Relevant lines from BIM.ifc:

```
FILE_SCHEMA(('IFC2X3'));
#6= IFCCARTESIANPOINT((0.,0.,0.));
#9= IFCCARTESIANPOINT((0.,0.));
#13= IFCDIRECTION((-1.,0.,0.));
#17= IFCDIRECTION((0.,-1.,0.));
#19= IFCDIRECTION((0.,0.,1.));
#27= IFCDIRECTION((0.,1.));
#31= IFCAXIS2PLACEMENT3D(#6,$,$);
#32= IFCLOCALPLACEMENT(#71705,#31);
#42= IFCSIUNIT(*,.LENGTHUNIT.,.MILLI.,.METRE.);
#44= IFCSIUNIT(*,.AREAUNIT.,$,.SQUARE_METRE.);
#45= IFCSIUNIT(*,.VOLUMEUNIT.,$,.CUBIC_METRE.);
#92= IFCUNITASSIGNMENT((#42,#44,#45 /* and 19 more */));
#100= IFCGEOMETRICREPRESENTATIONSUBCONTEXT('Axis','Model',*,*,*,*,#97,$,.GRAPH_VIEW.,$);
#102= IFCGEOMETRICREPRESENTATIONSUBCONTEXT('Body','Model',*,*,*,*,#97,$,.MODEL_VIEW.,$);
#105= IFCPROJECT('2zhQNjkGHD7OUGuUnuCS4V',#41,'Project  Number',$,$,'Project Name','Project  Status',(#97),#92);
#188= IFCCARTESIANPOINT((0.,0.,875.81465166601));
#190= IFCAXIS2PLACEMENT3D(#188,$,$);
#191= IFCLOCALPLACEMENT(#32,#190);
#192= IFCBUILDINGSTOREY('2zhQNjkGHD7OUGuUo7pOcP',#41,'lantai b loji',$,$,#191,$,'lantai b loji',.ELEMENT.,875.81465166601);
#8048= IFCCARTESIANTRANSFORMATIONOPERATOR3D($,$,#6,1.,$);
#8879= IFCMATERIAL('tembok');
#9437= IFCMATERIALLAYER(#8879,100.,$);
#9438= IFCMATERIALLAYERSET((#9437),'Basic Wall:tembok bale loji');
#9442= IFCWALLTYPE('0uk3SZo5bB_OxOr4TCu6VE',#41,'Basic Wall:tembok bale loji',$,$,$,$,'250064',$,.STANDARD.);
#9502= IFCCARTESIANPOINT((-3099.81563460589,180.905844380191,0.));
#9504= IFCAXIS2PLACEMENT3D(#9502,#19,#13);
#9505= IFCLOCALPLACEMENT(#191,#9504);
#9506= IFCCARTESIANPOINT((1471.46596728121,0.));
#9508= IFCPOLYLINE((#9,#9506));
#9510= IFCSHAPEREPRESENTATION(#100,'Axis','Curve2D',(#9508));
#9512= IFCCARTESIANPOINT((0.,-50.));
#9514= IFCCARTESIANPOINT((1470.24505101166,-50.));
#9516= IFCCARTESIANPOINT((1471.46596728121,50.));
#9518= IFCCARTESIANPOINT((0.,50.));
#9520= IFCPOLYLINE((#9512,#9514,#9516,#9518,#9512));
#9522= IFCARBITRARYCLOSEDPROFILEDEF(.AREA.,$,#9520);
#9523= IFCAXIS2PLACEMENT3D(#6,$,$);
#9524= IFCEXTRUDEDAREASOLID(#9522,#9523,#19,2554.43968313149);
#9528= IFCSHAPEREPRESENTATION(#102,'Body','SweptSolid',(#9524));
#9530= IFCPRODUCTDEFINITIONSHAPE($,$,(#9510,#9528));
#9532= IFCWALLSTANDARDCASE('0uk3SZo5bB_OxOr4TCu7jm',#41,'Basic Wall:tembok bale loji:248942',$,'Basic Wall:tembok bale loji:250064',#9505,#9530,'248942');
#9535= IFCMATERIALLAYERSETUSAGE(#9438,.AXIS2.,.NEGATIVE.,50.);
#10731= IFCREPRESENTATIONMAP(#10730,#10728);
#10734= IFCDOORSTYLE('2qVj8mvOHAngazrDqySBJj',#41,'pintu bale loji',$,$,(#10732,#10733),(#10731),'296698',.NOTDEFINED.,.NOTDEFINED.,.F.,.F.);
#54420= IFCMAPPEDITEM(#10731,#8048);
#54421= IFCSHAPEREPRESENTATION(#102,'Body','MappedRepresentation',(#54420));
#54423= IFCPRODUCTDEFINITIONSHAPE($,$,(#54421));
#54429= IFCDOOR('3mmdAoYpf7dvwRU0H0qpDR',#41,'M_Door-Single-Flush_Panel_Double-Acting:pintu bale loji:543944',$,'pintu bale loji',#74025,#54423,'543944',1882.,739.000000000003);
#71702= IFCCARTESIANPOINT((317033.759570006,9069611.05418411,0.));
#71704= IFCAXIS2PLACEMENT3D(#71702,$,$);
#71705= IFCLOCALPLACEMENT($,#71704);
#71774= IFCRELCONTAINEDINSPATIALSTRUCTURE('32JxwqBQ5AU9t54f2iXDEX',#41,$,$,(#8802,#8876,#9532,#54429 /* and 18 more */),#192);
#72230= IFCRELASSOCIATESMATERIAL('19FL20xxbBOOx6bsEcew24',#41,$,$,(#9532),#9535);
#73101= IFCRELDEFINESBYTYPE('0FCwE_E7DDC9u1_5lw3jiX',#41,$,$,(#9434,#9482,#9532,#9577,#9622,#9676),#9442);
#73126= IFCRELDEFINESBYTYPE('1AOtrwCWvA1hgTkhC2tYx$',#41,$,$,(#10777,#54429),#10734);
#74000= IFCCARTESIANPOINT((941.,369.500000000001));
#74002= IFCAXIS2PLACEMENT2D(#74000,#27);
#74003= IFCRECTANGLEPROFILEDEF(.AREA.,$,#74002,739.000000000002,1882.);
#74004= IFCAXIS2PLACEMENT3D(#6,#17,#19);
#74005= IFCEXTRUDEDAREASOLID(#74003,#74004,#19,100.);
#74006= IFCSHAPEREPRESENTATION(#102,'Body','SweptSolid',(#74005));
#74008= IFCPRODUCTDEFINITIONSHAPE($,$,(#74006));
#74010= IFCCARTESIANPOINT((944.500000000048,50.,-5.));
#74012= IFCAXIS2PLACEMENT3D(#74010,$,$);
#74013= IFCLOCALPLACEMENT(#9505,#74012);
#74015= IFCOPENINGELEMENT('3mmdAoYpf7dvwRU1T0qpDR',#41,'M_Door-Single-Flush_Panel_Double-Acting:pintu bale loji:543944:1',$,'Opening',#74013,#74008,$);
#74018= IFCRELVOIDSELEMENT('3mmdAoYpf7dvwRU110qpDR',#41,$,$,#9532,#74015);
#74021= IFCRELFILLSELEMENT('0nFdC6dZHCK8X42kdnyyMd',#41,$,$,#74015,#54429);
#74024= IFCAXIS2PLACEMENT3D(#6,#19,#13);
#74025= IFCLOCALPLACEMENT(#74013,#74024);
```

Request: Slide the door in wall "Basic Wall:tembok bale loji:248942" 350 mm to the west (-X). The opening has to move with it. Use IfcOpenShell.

```python
import ifcopenshell
import ifcopenshell.api.geometry
import ifcopenshell.util.placement
import ifcopenshell.util.unit

model = ifcopenshell.open("BIM.ifc")
unit_scale = ifcopenshell.util.unit.calculate_unit_scale(model)

door = model.by_id(54429)
opening = door.FillsVoids[0].RelatingOpeningElement
wall = opening.VoidsElements[0].RelatingBuildingElement

wall_matrix = ifcopenshell.util.placement.get_local_placement(wall.ObjectPlacement)
shift = wall_matrix[:3, 0] * 0.35 / unit_scale
before = ifcopenshell.util.placement.get_local_placement(door.ObjectPlacement)[:3, 3].copy()

# The door is placed relative to its opening, so it follows when the opening moves.
matrix = ifcopenshell.util.placement.get_local_placement(opening.ObjectPlacement)
matrix[:3, 3] += shift
ifcopenshell.api.geometry.edit_object_placement(
    model, product=opening, matrix=matrix, is_si=False, should_transform_children=True
)

after = ifcopenshell.util.placement.get_local_placement(door.ObjectPlacement)[:3, 3]
print("door moved by", (after - before).round(3) + 0.0)

model.write("BIM_v2.ifc")
```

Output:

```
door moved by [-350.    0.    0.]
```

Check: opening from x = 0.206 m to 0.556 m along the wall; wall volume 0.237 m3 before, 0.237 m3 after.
